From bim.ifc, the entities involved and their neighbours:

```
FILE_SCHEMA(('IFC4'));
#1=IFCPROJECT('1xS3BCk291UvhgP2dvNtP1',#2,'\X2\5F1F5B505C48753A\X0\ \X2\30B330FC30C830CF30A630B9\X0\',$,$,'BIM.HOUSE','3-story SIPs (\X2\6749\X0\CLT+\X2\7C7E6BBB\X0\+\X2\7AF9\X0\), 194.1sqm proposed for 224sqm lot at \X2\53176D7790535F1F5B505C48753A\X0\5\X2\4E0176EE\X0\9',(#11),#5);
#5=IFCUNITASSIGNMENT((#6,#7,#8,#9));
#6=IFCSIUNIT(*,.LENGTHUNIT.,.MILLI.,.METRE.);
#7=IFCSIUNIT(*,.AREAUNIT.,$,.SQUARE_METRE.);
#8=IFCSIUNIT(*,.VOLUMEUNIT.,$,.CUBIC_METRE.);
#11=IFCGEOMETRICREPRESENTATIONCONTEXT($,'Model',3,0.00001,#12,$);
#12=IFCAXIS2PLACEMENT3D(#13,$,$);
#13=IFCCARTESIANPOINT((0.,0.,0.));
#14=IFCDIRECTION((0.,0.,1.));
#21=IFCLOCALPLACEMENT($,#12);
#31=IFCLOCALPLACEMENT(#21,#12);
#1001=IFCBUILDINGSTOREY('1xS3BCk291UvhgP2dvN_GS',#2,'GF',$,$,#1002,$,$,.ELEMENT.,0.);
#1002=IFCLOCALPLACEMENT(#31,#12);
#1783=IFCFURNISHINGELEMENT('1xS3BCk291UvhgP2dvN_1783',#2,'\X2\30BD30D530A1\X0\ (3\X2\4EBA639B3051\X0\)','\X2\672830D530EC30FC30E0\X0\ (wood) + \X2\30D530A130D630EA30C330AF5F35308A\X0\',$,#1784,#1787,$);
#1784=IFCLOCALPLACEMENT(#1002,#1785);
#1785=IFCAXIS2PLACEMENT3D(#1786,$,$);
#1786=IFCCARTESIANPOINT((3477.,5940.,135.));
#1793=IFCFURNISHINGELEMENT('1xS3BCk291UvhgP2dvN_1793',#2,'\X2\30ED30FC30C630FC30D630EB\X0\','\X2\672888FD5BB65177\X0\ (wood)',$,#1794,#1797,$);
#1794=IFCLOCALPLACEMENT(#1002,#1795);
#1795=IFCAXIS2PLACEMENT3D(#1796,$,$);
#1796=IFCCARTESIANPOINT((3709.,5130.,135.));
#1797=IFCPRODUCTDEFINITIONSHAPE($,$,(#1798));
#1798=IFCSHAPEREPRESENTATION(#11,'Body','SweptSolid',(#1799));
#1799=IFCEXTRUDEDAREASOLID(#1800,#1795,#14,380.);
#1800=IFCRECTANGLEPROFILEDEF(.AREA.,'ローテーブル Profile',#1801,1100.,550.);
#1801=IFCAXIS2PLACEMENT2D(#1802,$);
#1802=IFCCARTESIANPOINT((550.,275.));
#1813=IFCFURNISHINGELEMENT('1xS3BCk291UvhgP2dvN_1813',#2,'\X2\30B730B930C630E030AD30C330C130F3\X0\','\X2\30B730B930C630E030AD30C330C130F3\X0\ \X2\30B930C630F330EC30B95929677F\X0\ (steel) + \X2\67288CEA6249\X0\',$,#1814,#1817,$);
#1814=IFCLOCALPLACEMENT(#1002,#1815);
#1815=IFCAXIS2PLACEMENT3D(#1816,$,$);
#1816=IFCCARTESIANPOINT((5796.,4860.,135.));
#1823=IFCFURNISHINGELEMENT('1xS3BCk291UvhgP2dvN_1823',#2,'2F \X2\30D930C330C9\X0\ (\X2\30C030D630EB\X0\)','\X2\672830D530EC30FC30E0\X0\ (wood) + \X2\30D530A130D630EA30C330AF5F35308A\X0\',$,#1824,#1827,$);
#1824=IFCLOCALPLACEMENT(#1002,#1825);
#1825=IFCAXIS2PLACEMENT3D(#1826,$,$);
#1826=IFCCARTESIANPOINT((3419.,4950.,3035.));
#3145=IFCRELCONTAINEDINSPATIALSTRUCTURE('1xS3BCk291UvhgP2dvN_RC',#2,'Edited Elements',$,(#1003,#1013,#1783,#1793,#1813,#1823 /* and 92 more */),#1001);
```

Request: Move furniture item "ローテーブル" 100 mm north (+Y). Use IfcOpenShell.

```python
import ifcopenshell
import ifcopenshell.api.geometry
import ifcopenshell.util.placement
import ifcopenshell.util.unit

model = ifcopenshell.open("bim.ifc")
unit_scale = ifcopenshell.util.unit.calculate_unit_scale(model)

item = model.by_guid("1xS3BCk291UvhgP2dvN_1793")
matrix = ifcopenshell.util.placement.get_local_placement(item.ObjectPlacement)
matrix[1, 3] += 0.1 / unit_scale
ifcopenshell.api.geometry.edit_object_placement(model, product=item, matrix=matrix, is_si=False)

print(ifcopenshell.util.placement.get_local_placement(item.ObjectPlacement).round(3) + 0.0)

model.write("bim_edited.ifc")
```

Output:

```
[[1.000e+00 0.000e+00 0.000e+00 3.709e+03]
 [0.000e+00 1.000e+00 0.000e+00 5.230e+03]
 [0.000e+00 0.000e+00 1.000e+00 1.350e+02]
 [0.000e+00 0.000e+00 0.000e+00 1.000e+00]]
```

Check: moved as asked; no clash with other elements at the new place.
